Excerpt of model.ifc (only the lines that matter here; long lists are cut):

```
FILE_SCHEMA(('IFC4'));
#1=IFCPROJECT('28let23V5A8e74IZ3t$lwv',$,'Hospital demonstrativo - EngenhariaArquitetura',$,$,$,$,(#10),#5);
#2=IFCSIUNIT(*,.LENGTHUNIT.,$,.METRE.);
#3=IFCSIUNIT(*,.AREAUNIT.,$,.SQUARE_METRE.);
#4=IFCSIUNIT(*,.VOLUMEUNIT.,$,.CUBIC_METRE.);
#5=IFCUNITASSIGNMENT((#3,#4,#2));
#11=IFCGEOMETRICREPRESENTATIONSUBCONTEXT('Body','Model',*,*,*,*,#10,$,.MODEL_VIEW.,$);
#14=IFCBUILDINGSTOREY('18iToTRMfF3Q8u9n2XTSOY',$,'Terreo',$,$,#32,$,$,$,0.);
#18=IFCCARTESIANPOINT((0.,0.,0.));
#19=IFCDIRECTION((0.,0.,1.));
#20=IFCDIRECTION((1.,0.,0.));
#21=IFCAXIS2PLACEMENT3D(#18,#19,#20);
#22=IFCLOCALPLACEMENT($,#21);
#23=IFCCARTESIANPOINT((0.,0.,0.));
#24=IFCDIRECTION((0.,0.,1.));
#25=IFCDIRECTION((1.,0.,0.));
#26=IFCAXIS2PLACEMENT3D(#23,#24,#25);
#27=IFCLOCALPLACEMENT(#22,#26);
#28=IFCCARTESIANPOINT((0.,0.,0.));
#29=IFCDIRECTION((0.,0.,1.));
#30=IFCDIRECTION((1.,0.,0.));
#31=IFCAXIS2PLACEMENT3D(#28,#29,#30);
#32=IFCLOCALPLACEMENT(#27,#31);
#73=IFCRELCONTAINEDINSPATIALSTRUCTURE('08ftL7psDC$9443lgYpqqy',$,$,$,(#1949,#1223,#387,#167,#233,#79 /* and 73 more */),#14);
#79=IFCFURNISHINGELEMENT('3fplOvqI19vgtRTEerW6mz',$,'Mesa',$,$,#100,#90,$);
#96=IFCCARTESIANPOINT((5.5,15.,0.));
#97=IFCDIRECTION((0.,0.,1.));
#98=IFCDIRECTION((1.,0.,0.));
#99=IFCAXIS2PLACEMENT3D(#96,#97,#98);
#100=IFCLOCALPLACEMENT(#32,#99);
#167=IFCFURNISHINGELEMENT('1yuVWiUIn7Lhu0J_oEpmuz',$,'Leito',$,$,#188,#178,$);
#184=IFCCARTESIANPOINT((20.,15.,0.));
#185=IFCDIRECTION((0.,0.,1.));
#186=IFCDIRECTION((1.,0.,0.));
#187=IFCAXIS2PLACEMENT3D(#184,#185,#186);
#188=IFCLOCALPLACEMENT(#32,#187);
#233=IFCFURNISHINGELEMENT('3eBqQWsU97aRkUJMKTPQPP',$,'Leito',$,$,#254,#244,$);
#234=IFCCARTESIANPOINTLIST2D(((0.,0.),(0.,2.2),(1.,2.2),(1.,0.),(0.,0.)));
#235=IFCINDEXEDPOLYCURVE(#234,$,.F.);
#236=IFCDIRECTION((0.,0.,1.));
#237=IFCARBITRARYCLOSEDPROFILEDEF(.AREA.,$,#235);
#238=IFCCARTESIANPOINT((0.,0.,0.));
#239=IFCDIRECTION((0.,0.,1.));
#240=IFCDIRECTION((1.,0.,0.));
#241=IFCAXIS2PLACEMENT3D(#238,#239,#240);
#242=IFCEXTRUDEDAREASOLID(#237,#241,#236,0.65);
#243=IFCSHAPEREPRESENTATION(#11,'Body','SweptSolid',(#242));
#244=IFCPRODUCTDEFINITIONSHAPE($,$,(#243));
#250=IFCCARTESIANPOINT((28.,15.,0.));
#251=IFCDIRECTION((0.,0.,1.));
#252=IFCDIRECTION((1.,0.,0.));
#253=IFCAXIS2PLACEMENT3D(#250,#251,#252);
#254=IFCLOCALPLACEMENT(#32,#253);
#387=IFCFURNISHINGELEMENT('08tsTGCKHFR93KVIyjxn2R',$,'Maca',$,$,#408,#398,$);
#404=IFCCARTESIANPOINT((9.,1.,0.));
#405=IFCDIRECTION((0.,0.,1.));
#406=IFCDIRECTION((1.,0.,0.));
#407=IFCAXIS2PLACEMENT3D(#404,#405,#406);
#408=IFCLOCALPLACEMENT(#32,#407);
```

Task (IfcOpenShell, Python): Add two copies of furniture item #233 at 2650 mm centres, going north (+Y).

```python
import numpy as np
import ifcopenshell
import ifcopenshell.api.geometry
import ifcopenshell.api.root
import ifcopenshell.util.element
import ifcopenshell.util.placement

model = ifcopenshell.open("model.ifc")

source = model.by_id(233)
base = ifcopenshell.util.placement.get_local_placement(source.ObjectPlacement)
step = np.array([0.0, 1.0, 0.0]) * 2.65

for i in range(1, 3):
    copy = ifcopenshell.api.root.copy_class(model, product=source)
    copy.Representation = ifcopenshell.util.element.copy_deep(
        model, source.Representation, exclude=["IfcGeometricRepresentationContext", "IfcRepresentationMap"]
    )
    matrix = base.copy()
    matrix[:3, 3] += i * step
    print("added at", matrix[:3, 3].round(3) + 0.0)
    ifcopenshell.api.geometry.edit_object_placement(model, product=copy, matrix=matrix, is_si=False)

model.write("model_v2.ifc")
```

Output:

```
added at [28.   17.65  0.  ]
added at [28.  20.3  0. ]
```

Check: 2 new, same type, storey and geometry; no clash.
